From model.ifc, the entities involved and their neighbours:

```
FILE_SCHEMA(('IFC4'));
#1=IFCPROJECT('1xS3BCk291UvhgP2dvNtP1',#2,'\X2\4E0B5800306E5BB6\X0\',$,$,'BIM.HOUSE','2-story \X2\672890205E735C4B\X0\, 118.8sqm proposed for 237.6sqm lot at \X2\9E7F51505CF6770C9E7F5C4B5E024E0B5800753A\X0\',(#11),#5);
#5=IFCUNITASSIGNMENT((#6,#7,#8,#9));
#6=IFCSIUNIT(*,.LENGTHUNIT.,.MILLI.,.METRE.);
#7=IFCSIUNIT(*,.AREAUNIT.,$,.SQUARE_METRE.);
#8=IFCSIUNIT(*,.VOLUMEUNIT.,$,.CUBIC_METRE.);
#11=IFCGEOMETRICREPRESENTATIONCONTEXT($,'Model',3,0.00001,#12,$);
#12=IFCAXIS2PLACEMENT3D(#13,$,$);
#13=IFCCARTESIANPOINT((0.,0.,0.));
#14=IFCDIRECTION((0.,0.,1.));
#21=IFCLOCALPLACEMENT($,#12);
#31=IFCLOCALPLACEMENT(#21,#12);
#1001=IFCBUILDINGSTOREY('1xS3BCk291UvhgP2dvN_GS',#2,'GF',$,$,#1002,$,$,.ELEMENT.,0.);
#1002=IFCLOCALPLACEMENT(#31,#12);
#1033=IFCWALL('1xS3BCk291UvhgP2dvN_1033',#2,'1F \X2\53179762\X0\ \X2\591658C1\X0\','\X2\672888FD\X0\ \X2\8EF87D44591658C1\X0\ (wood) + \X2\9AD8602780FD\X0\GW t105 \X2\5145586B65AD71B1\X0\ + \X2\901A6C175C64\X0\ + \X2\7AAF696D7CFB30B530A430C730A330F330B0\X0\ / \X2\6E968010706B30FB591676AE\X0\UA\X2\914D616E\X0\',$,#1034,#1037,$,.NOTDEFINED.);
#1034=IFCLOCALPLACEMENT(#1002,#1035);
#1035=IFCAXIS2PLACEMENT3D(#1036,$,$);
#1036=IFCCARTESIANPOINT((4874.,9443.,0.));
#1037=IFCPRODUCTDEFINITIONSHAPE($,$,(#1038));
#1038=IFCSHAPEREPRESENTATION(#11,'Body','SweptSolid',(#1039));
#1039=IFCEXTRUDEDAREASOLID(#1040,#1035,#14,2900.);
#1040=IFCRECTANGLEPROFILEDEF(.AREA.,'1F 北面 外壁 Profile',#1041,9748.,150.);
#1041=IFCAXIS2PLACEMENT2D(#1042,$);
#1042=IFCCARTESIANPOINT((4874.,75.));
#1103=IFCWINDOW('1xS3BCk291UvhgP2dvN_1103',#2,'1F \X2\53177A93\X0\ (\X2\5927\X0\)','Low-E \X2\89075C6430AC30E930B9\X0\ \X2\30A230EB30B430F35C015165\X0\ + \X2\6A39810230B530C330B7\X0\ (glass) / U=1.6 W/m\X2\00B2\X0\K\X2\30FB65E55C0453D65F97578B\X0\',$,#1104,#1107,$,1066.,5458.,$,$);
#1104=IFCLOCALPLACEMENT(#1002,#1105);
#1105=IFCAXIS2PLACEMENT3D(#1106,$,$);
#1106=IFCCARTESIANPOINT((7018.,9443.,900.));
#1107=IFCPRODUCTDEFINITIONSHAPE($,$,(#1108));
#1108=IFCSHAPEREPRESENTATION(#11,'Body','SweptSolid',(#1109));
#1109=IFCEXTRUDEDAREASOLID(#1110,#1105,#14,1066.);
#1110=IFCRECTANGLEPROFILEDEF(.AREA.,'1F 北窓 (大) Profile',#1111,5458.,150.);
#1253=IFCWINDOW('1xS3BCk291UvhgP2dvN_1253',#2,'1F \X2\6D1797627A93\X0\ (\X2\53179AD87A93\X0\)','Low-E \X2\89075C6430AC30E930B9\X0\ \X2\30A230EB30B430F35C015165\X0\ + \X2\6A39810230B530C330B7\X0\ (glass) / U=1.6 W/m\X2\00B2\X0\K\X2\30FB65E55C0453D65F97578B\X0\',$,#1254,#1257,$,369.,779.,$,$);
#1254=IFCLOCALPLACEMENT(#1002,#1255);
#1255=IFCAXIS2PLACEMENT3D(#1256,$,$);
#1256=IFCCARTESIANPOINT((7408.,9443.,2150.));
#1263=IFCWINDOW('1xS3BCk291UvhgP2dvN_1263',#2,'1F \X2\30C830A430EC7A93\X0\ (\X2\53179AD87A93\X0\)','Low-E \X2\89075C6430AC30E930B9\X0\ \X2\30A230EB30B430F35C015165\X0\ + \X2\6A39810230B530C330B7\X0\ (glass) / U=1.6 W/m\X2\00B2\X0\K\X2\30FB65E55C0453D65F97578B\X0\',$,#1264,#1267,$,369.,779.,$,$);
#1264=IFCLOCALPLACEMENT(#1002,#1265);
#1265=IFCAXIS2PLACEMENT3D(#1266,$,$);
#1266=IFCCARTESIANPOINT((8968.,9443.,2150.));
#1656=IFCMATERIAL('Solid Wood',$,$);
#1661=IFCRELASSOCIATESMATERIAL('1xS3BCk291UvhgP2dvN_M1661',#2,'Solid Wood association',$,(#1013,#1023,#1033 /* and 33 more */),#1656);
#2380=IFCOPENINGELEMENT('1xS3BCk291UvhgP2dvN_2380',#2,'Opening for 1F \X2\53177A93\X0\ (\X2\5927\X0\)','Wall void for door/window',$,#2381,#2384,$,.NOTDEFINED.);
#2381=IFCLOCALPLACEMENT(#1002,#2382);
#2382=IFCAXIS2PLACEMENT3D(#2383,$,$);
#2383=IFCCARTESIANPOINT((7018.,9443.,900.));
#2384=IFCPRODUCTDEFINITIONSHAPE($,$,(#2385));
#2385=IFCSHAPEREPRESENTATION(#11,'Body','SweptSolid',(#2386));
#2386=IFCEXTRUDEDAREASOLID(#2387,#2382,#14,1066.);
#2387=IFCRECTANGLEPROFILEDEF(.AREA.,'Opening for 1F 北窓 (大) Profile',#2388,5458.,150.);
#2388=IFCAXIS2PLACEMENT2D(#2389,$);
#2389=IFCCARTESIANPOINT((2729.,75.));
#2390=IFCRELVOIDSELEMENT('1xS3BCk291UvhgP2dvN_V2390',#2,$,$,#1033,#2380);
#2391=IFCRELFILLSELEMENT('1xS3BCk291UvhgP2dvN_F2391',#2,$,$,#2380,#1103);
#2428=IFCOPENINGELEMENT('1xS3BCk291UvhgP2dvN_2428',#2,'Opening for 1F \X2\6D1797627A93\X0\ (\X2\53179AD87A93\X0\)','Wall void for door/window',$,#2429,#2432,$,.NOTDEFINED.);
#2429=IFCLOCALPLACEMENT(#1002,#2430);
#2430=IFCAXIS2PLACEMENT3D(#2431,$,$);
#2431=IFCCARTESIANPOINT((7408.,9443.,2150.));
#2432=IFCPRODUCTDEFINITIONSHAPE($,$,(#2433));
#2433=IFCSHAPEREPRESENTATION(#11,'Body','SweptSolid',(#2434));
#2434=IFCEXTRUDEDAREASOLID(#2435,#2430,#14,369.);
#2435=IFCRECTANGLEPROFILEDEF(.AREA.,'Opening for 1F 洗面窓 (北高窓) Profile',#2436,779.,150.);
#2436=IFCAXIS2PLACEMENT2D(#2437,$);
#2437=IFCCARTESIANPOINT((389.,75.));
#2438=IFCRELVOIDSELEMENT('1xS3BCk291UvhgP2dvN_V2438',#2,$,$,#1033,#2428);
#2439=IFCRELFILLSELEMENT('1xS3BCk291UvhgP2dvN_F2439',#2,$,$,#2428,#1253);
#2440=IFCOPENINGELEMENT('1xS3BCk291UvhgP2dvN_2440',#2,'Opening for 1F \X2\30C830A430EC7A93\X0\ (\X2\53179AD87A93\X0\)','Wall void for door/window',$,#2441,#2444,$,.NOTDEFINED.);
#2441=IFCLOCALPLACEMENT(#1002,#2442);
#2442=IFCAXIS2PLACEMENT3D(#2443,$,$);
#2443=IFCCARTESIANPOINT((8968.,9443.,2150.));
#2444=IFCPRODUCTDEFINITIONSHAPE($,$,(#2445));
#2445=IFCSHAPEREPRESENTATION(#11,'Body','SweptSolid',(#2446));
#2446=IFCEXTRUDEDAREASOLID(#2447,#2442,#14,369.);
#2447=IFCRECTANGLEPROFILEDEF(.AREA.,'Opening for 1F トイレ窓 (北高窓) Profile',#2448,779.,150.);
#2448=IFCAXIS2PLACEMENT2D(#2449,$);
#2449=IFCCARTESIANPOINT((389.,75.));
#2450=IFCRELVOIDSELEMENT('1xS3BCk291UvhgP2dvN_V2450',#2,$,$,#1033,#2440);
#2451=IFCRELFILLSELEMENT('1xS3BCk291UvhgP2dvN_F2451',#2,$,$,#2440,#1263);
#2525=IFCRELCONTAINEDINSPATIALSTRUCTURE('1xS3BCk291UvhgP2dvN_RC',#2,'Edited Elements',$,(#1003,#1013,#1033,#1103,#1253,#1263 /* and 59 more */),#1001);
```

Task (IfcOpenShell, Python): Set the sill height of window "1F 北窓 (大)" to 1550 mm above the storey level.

```python
import numpy as np
import ifcopenshell
import ifcopenshell.api.geometry
import ifcopenshell.geom
import ifcopenshell.util.element
import ifcopenshell.util.placement
import ifcopenshell.util.shape
import ifcopenshell.util.unit

model = ifcopenshell.open("model.ifc")
unit_scale = ifcopenshell.util.unit.calculate_unit_scale(model)

window = model.by_id(1103)
opening = window.FillsVoids[0].RelatingOpeningElement
storey = ifcopenshell.util.element.get_container(window, ifc_class="IfcBuildingStorey")
level = ifcopenshell.util.placement.get_local_placement(storey.ObjectPlacement)[2, 3]

# The opening's origin need not be at the sill, so measure its lowest point.
shape = ifcopenshell.geom.create_shape(ifcopenshell.geom.settings(), opening)
bottom = ifcopenshell.util.shape.get_shape_bottom_elevation(shape, shape.geometry) / unit_scale
dz = level + 1.55 / unit_scale - bottom

shift = np.array([0.0, 0.0, dz])
# The window is not placed relative to its opening, so move both.
for product in (opening, window):
    matrix = ifcopenshell.util.placement.get_local_placement(product.ObjectPlacement)
    matrix[:3, 3] += shift
    ifcopenshell.api.geometry.edit_object_placement(model, product=product, matrix=matrix, is_si=False)

print(f"moved by {dz * unit_scale:+.3f} m")

model.write("model-out.ifc")
```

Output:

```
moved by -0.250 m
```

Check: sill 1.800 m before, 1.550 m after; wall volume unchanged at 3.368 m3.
